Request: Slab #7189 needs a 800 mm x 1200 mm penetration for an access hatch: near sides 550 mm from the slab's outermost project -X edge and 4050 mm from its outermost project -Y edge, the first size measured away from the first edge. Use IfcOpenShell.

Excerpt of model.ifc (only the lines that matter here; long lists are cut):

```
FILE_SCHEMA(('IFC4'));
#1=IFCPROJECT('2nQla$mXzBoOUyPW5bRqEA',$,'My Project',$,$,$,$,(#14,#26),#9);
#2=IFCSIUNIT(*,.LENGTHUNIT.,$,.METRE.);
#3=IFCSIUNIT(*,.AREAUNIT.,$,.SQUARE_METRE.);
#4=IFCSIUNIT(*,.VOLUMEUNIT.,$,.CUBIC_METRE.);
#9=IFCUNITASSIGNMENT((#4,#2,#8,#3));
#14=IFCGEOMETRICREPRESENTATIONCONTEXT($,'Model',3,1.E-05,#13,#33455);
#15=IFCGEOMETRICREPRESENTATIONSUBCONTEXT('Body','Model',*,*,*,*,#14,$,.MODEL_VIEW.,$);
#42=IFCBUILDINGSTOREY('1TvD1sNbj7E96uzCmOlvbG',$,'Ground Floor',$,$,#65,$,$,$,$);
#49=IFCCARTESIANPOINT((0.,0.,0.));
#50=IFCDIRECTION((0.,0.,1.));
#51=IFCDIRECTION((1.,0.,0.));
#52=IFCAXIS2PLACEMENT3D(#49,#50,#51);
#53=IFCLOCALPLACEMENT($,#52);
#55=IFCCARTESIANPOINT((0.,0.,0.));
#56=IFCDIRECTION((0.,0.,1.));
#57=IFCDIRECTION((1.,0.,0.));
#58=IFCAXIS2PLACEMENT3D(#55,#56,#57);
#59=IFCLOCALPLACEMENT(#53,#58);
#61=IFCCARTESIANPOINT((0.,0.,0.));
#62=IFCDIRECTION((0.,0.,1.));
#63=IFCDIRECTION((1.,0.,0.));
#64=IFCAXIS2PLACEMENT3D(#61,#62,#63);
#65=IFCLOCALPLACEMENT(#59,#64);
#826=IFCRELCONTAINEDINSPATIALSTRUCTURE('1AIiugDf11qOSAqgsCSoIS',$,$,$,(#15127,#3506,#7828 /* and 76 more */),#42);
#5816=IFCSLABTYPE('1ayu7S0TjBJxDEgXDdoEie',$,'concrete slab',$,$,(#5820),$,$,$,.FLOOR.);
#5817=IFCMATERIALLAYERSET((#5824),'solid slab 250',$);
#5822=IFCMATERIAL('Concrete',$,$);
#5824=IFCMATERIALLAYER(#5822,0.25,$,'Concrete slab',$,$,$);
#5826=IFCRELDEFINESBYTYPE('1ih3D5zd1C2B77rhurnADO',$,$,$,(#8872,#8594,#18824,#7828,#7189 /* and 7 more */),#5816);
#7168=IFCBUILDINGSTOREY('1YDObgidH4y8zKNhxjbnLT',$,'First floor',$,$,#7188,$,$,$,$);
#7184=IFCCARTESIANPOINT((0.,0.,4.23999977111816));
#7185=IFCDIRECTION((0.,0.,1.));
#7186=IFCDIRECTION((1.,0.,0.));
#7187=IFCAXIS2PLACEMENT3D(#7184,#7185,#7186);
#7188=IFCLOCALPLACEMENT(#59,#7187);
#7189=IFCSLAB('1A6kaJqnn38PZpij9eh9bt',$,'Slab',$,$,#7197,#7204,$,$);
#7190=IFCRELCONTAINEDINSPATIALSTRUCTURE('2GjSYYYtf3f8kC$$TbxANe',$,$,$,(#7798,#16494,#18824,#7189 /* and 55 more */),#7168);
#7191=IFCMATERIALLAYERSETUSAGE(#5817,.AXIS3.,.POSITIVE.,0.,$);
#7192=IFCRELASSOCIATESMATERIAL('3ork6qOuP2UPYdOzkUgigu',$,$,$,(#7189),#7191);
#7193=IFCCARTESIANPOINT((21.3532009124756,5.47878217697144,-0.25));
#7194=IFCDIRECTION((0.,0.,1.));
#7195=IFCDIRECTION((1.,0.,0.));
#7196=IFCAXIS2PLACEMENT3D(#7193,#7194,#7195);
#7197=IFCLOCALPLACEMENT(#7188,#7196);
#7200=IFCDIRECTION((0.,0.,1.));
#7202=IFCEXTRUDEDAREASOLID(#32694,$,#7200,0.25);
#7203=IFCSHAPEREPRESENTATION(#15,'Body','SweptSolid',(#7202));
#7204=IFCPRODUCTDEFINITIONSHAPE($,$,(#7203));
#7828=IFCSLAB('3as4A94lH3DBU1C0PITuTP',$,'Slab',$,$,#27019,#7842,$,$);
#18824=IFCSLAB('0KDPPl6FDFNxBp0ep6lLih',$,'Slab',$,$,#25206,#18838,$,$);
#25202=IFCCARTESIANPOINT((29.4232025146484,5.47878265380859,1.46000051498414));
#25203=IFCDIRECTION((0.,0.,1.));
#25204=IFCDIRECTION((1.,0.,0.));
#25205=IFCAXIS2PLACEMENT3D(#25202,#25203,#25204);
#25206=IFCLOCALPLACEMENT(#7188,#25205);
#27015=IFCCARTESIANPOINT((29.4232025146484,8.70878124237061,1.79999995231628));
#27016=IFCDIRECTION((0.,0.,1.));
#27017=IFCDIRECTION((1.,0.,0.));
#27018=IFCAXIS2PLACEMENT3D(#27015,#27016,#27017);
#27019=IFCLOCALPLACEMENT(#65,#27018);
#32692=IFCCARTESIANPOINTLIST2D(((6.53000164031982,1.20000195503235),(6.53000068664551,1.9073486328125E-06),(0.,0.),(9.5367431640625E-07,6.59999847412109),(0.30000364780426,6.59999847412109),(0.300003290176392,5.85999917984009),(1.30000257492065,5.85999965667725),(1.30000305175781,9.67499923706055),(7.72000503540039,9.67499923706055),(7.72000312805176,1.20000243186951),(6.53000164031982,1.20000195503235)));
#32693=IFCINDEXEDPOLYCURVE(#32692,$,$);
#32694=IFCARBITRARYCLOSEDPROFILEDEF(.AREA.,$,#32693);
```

```python
import numpy as np
import ifcopenshell
import ifcopenshell.api.feature
import ifcopenshell.api.geometry
import ifcopenshell.api.root
import ifcopenshell.geom
import ifcopenshell.util.placement
import ifcopenshell.util.representation
import ifcopenshell.util.shape
import ifcopenshell.util.unit

model = ifcopenshell.open("model.ifc")
unit_scale = ifcopenshell.util.unit.calculate_unit_scale(model)
settings = ifcopenshell.geom.settings()


def volume(element):
    """Net volume in cubic metres, openings subtracted."""
    shape = ifcopenshell.geom.create_shape(settings, element)
    return ifcopenshell.util.shape.get_volume(shape.geometry)


slab = model.by_guid("1A6kaJqnn38PZpij9eh9bt")
before = volume(slab)

# Extent in the slab's own axes, in metres. The edges named are its -X and -Y sides.
slab_shape = ifcopenshell.geom.create_shape(settings, slab)
vertices = ifcopenshell.util.shape.get_vertices(slab_shape.geometry)
x_min, y_min, bottom = vertices.min(axis=0)
top = vertices[:, 2].max()

opening = ifcopenshell.api.root.create_entity(model, ifc_class="IfcOpeningElement", name="Access hatch opening", predefined_type="OPENING")
context = ifcopenshell.util.representation.get_context(model, "Model", "Body", "MODEL_VIEW")
width, depth = 0.8, 1.2
outline = [(0.0, 0.0), (width, 0.0), (width, depth), (0.0, depth), (0.0, 0.0)]
# Overshoot both faces by 50 mm so the cut is clean.
shape = ifcopenshell.api.geometry.add_slab_representation(
    model, context=context, depth=top - bottom + 0.1, polyline=outline
)
ifcopenshell.api.geometry.assign_representation(model, product=opening, representation=shape)

matrix = ifcopenshell.util.placement.get_local_placement(slab.ObjectPlacement)
matrix[:, 3] = matrix @ np.append(np.array([x_min + 0.55, y_min + 4.05, bottom - 0.05]) / unit_scale, 1.0)
ifcopenshell.api.geometry.edit_object_placement(model, product=opening, matrix=matrix, is_si=False)
ifcopenshell.api.feature.add_feature(model, feature=opening, element=slab)

after = volume(slab)

print(f"slab volume {before:.3f} -> {after:.3f} m3")

model.write("model_rev.ifc")
```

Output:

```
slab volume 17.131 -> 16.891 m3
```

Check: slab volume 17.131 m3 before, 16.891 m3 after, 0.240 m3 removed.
